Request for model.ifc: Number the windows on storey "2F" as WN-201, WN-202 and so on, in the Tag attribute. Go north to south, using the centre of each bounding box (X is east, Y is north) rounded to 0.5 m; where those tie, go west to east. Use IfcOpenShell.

First a look at what the model holds.

```python
import ifcopenshell
import ifcopenshell.util.element
import ifcopenshell.util.placement

model = ifcopenshell.open("model.ifc")
print(model.schema)
storey = next(s for s in model.by_type("IfcBuildingStorey") if s.Name == "2F")
windows = [e for e in ifcopenshell.util.element.get_decomposition(storey) if e.is_a("IfcWindow")]
for e in sorted(windows, key=lambda e: e.id()):
    origin = ifcopenshell.util.placement.get_local_placement(e.ObjectPlacement)[:3, 3]
    print(e.id(), e.Tag, e.Name, origin.round(2) + 0.0, sep=" | ")
```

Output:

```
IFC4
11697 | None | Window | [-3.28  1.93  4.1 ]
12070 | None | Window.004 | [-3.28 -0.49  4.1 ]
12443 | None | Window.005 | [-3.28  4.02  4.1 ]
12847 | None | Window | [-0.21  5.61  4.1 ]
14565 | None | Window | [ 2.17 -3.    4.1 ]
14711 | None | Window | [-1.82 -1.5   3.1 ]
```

```python
import ifcopenshell
import ifcopenshell.geom
import ifcopenshell.util.element
import ifcopenshell.util.shape

model = ifcopenshell.open("model.ifc")
settings = ifcopenshell.geom.settings()
settings.set("use-world-coords", True)


def centre(element):
    shape = ifcopenshell.geom.create_shape(settings, element)
    return ifcopenshell.util.shape.get_bbox_centroid(shape.geometry)


storey = next(s for s in model.by_type("IfcBuildingStorey") if s.Name == "2F")
windows = [e for e in ifcopenshell.util.element.get_decomposition(storey) if e.is_a("IfcWindow")]

# Insertion points can sit at a corner or the storey origin, so sort by the geometry (in metres).
centres = {e: centre(e) for e in windows}
windows.sort(key=lambda e: (-round(centres[e][1] / 0.5), centres[e][0]))

for i, e in enumerate(windows, start=1):
    number = f"WN-2{i:02d}"
    e.Tag = number
    print(e.id(), number)

model.write("model_edited.ifc")
```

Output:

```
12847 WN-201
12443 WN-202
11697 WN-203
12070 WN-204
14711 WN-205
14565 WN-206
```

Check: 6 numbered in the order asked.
